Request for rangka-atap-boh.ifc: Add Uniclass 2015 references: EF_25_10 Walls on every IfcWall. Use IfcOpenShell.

First a look at what the model holds.

```python
import ifcopenshell

model = ifcopenshell.open("rangka-atap-boh.ifc")
print(model.schema)
print("classifications:", [c.Name for c in model.by_type("IfcClassification")])
for ifc_class in ("IfcDoor", "IfcRoof", "IfcStair", "IfcWall", "IfcWindow"):
    print(ifc_class, len(model.by_type(ifc_class)))
```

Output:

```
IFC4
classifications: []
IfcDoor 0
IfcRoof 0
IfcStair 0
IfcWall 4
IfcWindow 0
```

```python
import ifcopenshell
import ifcopenshell.api.classification

model = ifcopenshell.open("rangka-atap-boh.ifc")

system = ifcopenshell.api.classification.add_classification(model, classification="Uniclass 2015")

codes = {
    "IfcWall": ("EF_25_10", "Walls"),
}
for ifc_class, (code, name) in codes.items():
    products = model.by_type(ifc_class)
    ifcopenshell.api.classification.add_reference(
        model, products=products, classification=system, identification=code, name=name
    )
    print(code, len(products))

model.write("rangka-atap-boh_edited.ifc")
```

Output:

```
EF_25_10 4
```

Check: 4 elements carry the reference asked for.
